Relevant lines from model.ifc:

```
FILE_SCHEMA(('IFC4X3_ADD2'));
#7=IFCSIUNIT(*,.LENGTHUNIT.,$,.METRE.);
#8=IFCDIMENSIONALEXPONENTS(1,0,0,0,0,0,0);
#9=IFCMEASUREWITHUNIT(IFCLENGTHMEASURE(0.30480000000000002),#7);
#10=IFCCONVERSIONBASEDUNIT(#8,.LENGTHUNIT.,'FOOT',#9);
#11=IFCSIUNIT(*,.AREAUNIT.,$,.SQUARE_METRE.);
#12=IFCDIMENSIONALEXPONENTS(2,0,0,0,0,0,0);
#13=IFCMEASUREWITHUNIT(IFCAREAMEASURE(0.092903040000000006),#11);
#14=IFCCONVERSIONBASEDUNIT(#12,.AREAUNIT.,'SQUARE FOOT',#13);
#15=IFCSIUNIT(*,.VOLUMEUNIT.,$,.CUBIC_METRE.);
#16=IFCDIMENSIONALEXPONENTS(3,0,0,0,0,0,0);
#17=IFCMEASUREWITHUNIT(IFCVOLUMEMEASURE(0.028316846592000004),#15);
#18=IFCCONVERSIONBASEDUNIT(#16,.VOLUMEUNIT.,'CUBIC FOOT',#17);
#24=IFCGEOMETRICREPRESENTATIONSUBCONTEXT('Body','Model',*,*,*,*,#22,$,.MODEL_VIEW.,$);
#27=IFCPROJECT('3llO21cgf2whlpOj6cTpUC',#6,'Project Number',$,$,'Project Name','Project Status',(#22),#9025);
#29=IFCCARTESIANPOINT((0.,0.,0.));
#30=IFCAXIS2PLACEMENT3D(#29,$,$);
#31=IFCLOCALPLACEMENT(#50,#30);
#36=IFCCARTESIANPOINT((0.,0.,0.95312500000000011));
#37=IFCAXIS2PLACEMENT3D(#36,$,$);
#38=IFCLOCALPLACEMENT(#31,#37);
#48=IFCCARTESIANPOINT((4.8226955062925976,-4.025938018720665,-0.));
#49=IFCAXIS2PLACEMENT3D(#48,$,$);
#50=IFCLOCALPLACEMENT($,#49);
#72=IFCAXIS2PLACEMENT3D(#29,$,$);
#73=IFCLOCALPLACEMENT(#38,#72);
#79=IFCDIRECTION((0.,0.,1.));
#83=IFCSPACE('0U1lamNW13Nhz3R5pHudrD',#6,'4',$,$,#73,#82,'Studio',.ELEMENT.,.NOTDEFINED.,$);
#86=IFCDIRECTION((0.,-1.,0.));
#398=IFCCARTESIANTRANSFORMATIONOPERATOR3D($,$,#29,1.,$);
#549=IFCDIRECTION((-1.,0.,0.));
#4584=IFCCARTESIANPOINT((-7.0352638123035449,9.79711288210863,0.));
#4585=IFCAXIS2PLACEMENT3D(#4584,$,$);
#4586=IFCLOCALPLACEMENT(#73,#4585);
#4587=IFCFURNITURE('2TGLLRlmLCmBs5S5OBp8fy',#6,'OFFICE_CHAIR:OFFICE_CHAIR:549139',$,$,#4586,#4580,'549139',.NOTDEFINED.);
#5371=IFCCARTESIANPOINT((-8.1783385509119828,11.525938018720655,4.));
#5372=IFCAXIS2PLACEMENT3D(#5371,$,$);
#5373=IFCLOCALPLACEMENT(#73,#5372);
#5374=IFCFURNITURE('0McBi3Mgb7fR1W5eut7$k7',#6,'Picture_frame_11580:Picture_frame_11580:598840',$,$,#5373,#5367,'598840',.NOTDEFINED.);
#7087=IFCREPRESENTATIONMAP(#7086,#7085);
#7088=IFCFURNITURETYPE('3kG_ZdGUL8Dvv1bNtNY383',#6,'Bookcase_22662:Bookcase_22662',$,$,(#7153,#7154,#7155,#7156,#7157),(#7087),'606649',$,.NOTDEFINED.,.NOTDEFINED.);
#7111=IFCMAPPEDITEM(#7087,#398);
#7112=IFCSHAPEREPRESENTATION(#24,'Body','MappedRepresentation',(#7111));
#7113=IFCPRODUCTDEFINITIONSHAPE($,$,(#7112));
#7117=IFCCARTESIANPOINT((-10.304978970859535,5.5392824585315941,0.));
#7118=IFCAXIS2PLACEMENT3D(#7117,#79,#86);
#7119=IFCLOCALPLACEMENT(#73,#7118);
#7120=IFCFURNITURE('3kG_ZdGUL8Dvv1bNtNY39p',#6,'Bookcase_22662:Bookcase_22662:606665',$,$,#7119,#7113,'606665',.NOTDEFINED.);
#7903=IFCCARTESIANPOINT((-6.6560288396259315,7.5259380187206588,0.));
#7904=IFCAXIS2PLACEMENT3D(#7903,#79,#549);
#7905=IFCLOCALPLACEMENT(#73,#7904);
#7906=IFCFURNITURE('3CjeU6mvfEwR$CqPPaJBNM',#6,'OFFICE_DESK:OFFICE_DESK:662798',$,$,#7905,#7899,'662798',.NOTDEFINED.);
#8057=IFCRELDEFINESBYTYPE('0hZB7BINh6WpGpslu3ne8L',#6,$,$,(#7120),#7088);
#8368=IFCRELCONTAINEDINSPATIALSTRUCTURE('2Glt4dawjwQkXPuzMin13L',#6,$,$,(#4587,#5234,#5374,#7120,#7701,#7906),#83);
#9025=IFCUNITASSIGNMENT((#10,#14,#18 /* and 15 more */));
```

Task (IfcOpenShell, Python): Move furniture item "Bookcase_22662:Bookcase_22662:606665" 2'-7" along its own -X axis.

```python
import ifcopenshell
import ifcopenshell.api.geometry
import ifcopenshell.util.placement
import ifcopenshell.util.unit

model = ifcopenshell.open("model.ifc")
unit_scale = ifcopenshell.util.unit.calculate_unit_scale(model)

item = model.by_id(7120)
matrix = ifcopenshell.util.placement.get_local_placement(item.ObjectPlacement)
matrix[:3, 3] -= matrix[:3, 0] * 31 * 0.0254 / unit_scale
ifcopenshell.api.geometry.edit_object_placement(model, product=item, matrix=matrix, is_si=False)

print(ifcopenshell.util.placement.get_local_placement(item.ObjectPlacement).round(3) + 0.0)

model.write("model_edited.ifc")
```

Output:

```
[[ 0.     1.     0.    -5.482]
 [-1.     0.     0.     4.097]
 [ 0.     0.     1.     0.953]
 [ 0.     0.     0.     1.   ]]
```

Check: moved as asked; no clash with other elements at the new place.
